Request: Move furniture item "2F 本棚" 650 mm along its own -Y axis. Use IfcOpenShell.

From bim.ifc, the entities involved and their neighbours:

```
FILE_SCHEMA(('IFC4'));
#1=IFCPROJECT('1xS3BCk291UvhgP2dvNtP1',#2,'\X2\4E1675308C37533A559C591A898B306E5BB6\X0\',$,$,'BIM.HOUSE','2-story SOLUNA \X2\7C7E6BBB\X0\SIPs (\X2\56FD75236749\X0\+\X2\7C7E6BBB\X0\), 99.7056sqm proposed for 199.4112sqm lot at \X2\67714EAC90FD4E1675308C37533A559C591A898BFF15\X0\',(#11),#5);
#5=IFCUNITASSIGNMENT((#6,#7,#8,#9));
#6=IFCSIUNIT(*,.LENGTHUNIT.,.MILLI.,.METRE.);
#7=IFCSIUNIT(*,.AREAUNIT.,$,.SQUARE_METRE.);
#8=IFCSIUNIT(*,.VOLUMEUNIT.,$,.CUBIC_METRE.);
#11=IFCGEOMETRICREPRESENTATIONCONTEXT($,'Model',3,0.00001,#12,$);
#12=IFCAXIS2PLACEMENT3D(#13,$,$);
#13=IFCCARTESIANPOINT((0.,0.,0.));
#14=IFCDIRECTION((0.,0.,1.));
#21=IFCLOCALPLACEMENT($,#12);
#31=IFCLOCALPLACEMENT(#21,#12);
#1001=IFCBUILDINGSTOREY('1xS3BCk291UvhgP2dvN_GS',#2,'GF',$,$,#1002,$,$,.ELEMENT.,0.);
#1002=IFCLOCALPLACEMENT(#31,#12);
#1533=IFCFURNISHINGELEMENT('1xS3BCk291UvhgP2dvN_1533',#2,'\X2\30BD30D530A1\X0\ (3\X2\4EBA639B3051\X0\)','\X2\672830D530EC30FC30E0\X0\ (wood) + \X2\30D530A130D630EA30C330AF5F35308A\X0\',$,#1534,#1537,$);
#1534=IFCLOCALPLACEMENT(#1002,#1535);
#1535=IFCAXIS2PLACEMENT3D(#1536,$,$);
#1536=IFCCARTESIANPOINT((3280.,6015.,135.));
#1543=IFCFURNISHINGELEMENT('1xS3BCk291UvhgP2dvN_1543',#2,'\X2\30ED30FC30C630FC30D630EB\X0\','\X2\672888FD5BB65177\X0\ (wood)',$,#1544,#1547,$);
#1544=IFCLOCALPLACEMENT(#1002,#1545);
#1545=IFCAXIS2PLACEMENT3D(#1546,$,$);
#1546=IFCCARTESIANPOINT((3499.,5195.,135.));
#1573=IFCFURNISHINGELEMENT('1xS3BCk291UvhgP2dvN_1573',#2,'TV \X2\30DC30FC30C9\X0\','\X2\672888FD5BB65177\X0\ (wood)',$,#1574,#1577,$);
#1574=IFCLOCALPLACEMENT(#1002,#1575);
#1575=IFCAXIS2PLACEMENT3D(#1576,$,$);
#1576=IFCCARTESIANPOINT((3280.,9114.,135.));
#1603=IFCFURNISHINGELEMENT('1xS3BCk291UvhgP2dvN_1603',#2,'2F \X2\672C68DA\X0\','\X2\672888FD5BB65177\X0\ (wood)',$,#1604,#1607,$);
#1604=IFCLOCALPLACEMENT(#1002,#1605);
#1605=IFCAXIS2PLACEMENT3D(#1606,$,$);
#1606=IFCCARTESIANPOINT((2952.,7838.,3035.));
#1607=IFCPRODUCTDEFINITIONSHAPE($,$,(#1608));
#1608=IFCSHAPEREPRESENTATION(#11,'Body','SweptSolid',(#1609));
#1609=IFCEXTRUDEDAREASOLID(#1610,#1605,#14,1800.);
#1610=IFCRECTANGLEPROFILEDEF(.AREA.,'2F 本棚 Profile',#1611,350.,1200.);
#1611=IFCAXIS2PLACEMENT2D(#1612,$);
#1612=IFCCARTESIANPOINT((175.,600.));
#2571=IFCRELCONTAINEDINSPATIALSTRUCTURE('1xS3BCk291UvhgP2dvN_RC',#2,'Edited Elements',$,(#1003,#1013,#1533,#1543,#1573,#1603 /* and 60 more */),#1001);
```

```python
import ifcopenshell
import ifcopenshell.api.geometry
import ifcopenshell.util.placement
import ifcopenshell.util.unit

model = ifcopenshell.open("bim.ifc")
unit_scale = ifcopenshell.util.unit.calculate_unit_scale(model)

item = model.by_guid("1xS3BCk291UvhgP2dvN_1603")
matrix = ifcopenshell.util.placement.get_local_placement(item.ObjectPlacement)
matrix[:3, 3] -= matrix[:3, 1] * 0.65 / unit_scale
ifcopenshell.api.geometry.edit_object_placement(model, product=item, matrix=matrix, is_si=False)

print(ifcopenshell.util.placement.get_local_placement(item.ObjectPlacement).round(3) + 0.0)

model.write("bim_updated.ifc")
```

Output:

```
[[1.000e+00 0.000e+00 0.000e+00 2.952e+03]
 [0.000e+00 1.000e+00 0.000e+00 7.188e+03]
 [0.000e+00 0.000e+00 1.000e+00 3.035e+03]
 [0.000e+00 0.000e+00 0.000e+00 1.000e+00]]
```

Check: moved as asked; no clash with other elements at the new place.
